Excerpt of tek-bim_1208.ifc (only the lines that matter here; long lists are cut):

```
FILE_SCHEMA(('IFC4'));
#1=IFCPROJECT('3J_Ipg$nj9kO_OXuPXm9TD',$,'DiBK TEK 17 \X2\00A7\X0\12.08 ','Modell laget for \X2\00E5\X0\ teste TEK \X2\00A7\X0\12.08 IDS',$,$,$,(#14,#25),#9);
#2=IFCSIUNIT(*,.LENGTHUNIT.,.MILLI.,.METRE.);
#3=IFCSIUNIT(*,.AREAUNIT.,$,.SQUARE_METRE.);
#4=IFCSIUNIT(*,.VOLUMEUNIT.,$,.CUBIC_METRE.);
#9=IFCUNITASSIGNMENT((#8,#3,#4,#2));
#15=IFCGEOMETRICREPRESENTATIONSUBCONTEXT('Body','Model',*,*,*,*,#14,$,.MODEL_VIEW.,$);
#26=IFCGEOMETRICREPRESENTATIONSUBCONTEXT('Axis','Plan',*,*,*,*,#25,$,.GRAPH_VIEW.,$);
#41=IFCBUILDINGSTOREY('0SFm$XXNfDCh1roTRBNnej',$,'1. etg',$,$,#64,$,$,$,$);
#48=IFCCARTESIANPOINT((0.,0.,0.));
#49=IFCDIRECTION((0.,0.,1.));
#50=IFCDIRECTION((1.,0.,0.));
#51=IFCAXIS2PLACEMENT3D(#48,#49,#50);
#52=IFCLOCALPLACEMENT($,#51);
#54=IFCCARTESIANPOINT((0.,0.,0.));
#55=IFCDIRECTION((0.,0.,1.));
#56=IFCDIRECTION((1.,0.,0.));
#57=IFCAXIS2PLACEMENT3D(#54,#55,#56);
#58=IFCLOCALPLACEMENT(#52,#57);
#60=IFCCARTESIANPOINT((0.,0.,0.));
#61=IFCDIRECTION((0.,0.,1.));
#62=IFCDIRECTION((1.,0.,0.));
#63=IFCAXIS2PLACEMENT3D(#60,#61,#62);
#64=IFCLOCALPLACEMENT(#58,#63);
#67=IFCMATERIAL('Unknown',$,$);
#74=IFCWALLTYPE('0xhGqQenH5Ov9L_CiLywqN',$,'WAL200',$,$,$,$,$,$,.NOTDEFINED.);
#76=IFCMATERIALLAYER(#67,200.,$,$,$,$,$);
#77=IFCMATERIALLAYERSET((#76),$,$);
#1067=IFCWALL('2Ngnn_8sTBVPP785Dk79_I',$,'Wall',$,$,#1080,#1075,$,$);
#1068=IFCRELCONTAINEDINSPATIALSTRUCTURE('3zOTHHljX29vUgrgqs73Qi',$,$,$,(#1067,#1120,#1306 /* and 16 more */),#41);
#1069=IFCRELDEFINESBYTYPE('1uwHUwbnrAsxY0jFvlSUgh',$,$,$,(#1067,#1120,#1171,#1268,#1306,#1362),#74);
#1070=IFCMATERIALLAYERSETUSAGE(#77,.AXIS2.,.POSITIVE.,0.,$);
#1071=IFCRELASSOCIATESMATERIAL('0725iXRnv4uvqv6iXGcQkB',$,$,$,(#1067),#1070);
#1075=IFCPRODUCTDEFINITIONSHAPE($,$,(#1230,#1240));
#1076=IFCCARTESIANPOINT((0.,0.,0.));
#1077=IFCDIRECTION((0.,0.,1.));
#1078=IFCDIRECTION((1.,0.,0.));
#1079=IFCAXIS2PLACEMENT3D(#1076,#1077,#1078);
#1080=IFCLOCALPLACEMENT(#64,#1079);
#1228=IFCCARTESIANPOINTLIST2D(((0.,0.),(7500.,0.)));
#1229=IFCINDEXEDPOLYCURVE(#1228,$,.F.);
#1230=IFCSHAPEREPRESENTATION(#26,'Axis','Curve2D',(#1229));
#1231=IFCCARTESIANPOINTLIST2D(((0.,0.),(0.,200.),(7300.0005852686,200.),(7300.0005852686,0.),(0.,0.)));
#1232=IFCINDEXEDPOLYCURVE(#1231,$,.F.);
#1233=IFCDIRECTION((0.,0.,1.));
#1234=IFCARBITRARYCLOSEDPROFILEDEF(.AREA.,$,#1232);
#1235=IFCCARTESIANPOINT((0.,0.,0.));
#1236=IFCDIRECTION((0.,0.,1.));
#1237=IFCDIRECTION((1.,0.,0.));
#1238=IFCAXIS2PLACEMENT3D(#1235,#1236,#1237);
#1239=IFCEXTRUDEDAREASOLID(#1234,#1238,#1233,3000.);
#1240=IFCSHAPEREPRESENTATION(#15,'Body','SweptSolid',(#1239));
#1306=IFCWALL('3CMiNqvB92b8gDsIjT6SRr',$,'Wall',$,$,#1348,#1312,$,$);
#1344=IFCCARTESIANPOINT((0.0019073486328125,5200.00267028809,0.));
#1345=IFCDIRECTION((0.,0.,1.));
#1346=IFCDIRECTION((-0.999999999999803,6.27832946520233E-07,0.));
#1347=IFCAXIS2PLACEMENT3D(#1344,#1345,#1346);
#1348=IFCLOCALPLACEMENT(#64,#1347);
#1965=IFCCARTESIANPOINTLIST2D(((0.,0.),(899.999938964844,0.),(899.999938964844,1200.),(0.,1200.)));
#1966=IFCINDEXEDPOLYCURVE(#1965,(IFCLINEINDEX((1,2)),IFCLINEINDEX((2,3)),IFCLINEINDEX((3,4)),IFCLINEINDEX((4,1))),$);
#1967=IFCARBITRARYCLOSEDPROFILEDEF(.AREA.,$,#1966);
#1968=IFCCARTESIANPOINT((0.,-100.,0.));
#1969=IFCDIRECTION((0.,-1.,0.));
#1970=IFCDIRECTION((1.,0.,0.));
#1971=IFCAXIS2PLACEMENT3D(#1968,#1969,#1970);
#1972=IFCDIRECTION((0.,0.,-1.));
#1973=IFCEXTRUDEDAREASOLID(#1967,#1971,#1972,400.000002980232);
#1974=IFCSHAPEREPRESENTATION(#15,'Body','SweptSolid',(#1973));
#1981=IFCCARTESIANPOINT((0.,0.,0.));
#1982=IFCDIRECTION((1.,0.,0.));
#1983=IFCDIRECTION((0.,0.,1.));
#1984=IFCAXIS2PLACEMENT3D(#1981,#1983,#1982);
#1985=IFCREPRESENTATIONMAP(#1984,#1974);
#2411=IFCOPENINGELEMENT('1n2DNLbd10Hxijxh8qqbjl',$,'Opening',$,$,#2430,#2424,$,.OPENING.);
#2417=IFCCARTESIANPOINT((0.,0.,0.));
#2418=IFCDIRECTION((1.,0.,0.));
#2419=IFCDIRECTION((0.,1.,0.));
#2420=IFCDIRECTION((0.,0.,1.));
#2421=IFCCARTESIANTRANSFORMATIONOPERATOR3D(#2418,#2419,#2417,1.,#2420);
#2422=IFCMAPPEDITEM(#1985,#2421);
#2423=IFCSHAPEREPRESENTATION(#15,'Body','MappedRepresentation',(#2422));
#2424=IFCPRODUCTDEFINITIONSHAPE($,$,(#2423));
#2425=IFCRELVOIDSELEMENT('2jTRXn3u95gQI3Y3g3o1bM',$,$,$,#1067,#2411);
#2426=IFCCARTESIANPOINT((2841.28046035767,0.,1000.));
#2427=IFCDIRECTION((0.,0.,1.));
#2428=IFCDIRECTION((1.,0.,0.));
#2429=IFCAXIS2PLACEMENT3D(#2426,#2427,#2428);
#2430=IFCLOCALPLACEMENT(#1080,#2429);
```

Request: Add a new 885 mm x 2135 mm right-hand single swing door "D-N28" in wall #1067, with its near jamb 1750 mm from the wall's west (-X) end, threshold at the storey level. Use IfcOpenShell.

```python
import numpy as np
import ifcopenshell
import ifcopenshell.api.feature
import ifcopenshell.api.geometry
import ifcopenshell.api.root
import ifcopenshell.api.spatial
import ifcopenshell.geom
import ifcopenshell.util.element
import ifcopenshell.util.placement
import ifcopenshell.util.representation
import ifcopenshell.util.shape
import ifcopenshell.util.unit

model = ifcopenshell.open("tek-bim_1208.ifc")
unit_scale = ifcopenshell.util.unit.calculate_unit_scale(model)
settings = ifcopenshell.geom.settings()


def volume(element):
    """Net volume in cubic metres, openings subtracted."""
    shape = ifcopenshell.geom.create_shape(settings, element)
    return ifcopenshell.util.shape.get_volume(shape.geometry)


wall = model.by_guid("2Ngnn_8sTBVPP785Dk79_I")
storey = ifcopenshell.util.element.get_container(wall, ifc_class="IfcBuildingStorey")
context = ifcopenshell.util.representation.get_context(model, "Model", "Body", "MODEL_VIEW")
before = volume(wall)

width, height, from_end, sill = 0.885, 2.135, 1.75, 0.0  # metres

# The wall runs along its own X axis, and the end named is its -X end.
wall_shape = ifcopenshell.geom.create_shape(settings, wall)
x, y, z = ifcopenshell.util.shape.get_vertices(wall_shape.geometry).T
start = x.min() + from_end
face, thickness = float(y.min()), float(y.max() - y.min())
wall_matrix = ifcopenshell.util.placement.get_local_placement(wall.ObjectPlacement)
level = ifcopenshell.util.placement.get_local_placement(storey.ObjectPlacement)[2, 3]


def in_wall(x, y):
    """Placement at x, y metres in the wall's axes, at sill height."""
    matrix = wall_matrix.copy()
    matrix[:, 3] = wall_matrix @ np.array([x / unit_scale, y / unit_scale, 0.0, 1.0])
    matrix[2, 3] = level + sill / unit_scale
    return matrix


# Opening: a box that overshoots both wall faces by 50 mm.
opening = ifcopenshell.api.root.create_entity(model, ifc_class="IfcOpeningElement", predefined_type="OPENING")
box = ifcopenshell.api.geometry.add_wall_representation(
    model, context=context, length=width, height=height, thickness=thickness + 0.1
)
ifcopenshell.api.geometry.assign_representation(model, product=opening, representation=box)
ifcopenshell.api.geometry.edit_object_placement(model, product=opening, matrix=in_wall(start, face - 0.05), is_si=False)
ifcopenshell.api.feature.add_feature(model, feature=opening, element=wall)

door = ifcopenshell.api.root.create_entity(model, ifc_class="IfcDoor", name="D-N28", predefined_type="DOOR")
door.OverallWidth, door.OverallHeight = width / unit_scale, height / unit_scale
door.OperationType = "SINGLE_SWING_RIGHT"
body = ifcopenshell.api.geometry.add_door_representation(
    model,
    context=context,
    overall_width=door.OverallWidth,
    overall_height=door.OverallHeight,
    operation_type="SINGLE_SWING_RIGHT",
    lining_properties={"LiningDepth": thickness / unit_scale, "ThresholdDepth": thickness / unit_scale},
)
ifcopenshell.api.geometry.assign_representation(model, product=door, representation=body)
ifcopenshell.api.spatial.assign_container(model, products=[door], relating_structure=storey)
ifcopenshell.api.feature.add_filling(model, opening=opening, element=door)

# The lining spans the wall, so the door starts at the wall face.
ifcopenshell.api.geometry.edit_object_placement(model, product=door, matrix=in_wall(start, face), is_si=False)

after = volume(wall)

print(f"wall volume {before:.3f} -> {after:.3f} m3")

model.write("tek-bim_1208_rev.ifc")
```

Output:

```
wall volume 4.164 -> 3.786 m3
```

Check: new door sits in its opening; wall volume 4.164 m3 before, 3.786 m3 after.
